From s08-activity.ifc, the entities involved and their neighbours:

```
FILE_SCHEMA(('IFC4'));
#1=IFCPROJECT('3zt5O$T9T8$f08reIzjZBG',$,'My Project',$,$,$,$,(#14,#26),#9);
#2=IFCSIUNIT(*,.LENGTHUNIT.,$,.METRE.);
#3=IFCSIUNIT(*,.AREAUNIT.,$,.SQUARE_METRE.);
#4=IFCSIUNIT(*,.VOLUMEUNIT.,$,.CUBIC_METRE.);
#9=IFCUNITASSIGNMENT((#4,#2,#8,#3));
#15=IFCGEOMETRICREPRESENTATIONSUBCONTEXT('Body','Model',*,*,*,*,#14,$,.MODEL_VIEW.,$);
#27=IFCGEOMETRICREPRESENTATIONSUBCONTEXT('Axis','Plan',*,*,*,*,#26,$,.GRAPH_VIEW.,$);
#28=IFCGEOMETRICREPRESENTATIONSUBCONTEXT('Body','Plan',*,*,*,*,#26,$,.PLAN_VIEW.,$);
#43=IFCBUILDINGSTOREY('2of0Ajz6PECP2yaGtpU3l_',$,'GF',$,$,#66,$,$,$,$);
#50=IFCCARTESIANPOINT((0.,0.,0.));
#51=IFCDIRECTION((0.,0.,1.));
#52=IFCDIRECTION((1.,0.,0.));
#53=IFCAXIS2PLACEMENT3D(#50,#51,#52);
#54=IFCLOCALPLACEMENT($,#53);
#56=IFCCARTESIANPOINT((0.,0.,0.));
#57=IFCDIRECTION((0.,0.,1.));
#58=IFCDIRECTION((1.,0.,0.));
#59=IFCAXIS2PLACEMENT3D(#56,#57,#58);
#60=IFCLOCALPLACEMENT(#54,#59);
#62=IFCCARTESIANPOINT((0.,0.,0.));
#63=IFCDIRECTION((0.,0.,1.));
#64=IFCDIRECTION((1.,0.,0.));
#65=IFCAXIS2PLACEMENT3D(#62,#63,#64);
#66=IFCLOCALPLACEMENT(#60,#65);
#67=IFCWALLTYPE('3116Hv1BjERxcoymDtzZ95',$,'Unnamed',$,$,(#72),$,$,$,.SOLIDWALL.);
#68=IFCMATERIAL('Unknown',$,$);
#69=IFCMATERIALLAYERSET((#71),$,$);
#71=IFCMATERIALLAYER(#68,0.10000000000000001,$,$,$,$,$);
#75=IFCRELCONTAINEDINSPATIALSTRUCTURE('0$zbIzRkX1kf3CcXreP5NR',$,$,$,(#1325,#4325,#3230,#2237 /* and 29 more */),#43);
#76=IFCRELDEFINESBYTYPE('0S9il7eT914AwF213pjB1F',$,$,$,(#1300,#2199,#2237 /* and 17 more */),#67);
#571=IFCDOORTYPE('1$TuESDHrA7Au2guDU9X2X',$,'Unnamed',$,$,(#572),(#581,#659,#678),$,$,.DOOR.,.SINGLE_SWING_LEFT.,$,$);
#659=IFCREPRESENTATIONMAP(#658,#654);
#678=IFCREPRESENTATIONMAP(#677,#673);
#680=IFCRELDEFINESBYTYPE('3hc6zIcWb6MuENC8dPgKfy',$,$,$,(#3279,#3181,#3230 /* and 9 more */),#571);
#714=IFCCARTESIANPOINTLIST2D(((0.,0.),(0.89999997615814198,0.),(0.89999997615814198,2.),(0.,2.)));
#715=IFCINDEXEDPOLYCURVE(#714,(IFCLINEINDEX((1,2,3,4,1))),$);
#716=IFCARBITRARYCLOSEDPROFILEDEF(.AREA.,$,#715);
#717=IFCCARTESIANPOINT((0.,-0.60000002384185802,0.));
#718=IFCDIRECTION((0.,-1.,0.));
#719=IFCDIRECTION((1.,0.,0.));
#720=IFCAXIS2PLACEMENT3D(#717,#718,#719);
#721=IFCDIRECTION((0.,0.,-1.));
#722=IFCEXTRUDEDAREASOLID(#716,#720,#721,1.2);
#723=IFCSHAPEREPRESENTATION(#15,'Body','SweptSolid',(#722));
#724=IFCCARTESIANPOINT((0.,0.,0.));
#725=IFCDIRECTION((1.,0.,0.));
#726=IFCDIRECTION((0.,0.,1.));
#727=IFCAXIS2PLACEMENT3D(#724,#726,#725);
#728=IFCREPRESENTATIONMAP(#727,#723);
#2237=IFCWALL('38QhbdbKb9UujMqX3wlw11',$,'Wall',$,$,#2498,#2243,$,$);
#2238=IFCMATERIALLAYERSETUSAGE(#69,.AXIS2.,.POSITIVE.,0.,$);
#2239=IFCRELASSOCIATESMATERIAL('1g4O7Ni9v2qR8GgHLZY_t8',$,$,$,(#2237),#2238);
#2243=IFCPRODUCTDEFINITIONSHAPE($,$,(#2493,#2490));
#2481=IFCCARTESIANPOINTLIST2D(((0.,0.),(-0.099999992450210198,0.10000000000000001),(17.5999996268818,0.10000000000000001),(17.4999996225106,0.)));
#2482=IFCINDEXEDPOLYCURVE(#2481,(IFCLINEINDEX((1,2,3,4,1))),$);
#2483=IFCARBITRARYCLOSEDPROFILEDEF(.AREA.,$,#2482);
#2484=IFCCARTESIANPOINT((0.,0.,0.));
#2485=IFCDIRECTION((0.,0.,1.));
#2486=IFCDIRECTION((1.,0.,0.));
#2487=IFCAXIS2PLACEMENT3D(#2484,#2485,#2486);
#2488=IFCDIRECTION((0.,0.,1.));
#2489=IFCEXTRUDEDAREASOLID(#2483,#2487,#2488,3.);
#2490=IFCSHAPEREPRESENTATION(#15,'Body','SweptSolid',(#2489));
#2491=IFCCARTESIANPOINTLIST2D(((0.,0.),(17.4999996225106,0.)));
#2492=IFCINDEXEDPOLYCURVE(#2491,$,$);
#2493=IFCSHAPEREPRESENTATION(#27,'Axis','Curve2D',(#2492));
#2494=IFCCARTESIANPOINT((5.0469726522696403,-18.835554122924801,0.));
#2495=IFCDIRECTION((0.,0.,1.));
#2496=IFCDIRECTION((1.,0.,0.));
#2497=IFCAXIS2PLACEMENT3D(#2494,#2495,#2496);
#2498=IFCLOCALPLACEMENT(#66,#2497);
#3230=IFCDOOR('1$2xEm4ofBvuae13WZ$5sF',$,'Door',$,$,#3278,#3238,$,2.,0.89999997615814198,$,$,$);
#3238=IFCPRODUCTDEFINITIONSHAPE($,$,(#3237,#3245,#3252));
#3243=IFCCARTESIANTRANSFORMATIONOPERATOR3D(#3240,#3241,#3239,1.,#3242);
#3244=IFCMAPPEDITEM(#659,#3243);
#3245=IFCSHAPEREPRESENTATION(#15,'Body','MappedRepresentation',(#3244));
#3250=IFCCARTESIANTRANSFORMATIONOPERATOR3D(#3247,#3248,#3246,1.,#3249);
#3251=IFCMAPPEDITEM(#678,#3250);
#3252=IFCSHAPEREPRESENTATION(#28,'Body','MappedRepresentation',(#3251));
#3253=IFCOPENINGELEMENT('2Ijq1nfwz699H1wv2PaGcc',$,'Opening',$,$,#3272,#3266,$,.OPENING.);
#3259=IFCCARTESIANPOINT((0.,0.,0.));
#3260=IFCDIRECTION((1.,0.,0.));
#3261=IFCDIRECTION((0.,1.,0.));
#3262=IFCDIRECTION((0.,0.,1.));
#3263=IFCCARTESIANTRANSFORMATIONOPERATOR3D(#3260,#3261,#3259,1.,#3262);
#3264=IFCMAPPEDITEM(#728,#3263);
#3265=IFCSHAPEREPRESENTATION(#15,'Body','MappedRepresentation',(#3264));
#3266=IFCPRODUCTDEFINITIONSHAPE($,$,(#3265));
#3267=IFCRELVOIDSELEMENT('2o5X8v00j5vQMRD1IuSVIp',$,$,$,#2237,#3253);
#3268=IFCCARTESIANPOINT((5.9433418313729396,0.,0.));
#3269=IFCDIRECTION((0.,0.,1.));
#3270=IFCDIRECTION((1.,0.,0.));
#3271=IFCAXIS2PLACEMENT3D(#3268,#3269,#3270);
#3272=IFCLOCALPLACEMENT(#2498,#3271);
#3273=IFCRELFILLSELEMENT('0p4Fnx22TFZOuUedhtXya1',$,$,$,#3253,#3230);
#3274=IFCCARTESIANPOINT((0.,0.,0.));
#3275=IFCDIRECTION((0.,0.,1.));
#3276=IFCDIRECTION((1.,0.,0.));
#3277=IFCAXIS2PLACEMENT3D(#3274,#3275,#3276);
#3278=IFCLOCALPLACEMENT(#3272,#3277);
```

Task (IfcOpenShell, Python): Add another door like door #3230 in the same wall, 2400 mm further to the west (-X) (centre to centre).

```python
import ifcopenshell
import ifcopenshell.api.feature
import ifcopenshell.api.geometry
import ifcopenshell.api.root
import ifcopenshell.geom
import ifcopenshell.util.element
import ifcopenshell.util.placement
import ifcopenshell.util.shape

model = ifcopenshell.open("s08-activity.ifc")
settings = ifcopenshell.geom.settings()


def volume(element):
    """Net volume in cubic metres, openings subtracted."""
    shape = ifcopenshell.geom.create_shape(settings, element)
    return ifcopenshell.util.shape.get_volume(shape.geometry)


door = model.by_id(3230)
opening = door.FillsVoids[0].RelatingOpeningElement
wall = opening.VoidsElements[0].RelatingBuildingElement
before = volume(wall)
shift = ifcopenshell.util.placement.get_local_placement(wall.ObjectPlacement)[:3, 0] * -2.4

# copy_class copies the void relationship, type, container and properties, but no geometry.
new_opening = ifcopenshell.api.root.copy_class(model, product=opening)
new_opening.Representation = ifcopenshell.util.element.copy_deep(
    model, opening.Representation, exclude=["IfcGeometricRepresentationContext", "IfcRepresentationMap"]
)
new_door = ifcopenshell.api.root.copy_class(model, product=door)
new_door.Representation = ifcopenshell.util.element.copy_deep(
    model, door.Representation, exclude=["IfcGeometricRepresentationContext", "IfcRepresentationMap"]
)
ifcopenshell.api.feature.add_filling(model, opening=new_opening, element=new_door)

for old, new in ((opening, new_opening), (door, new_door)):
    matrix = ifcopenshell.util.placement.get_local_placement(old.ObjectPlacement)
    matrix[:3, 3] += shift
    ifcopenshell.api.geometry.edit_object_placement(model, product=new, matrix=matrix, is_si=False)

after = volume(wall)

print(f"wall volume {before:.3f} -> {after:.3f} m3")

model.write("s08-activity_updated.ifc")
```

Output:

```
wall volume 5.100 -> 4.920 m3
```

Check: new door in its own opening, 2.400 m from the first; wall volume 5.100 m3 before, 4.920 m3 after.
